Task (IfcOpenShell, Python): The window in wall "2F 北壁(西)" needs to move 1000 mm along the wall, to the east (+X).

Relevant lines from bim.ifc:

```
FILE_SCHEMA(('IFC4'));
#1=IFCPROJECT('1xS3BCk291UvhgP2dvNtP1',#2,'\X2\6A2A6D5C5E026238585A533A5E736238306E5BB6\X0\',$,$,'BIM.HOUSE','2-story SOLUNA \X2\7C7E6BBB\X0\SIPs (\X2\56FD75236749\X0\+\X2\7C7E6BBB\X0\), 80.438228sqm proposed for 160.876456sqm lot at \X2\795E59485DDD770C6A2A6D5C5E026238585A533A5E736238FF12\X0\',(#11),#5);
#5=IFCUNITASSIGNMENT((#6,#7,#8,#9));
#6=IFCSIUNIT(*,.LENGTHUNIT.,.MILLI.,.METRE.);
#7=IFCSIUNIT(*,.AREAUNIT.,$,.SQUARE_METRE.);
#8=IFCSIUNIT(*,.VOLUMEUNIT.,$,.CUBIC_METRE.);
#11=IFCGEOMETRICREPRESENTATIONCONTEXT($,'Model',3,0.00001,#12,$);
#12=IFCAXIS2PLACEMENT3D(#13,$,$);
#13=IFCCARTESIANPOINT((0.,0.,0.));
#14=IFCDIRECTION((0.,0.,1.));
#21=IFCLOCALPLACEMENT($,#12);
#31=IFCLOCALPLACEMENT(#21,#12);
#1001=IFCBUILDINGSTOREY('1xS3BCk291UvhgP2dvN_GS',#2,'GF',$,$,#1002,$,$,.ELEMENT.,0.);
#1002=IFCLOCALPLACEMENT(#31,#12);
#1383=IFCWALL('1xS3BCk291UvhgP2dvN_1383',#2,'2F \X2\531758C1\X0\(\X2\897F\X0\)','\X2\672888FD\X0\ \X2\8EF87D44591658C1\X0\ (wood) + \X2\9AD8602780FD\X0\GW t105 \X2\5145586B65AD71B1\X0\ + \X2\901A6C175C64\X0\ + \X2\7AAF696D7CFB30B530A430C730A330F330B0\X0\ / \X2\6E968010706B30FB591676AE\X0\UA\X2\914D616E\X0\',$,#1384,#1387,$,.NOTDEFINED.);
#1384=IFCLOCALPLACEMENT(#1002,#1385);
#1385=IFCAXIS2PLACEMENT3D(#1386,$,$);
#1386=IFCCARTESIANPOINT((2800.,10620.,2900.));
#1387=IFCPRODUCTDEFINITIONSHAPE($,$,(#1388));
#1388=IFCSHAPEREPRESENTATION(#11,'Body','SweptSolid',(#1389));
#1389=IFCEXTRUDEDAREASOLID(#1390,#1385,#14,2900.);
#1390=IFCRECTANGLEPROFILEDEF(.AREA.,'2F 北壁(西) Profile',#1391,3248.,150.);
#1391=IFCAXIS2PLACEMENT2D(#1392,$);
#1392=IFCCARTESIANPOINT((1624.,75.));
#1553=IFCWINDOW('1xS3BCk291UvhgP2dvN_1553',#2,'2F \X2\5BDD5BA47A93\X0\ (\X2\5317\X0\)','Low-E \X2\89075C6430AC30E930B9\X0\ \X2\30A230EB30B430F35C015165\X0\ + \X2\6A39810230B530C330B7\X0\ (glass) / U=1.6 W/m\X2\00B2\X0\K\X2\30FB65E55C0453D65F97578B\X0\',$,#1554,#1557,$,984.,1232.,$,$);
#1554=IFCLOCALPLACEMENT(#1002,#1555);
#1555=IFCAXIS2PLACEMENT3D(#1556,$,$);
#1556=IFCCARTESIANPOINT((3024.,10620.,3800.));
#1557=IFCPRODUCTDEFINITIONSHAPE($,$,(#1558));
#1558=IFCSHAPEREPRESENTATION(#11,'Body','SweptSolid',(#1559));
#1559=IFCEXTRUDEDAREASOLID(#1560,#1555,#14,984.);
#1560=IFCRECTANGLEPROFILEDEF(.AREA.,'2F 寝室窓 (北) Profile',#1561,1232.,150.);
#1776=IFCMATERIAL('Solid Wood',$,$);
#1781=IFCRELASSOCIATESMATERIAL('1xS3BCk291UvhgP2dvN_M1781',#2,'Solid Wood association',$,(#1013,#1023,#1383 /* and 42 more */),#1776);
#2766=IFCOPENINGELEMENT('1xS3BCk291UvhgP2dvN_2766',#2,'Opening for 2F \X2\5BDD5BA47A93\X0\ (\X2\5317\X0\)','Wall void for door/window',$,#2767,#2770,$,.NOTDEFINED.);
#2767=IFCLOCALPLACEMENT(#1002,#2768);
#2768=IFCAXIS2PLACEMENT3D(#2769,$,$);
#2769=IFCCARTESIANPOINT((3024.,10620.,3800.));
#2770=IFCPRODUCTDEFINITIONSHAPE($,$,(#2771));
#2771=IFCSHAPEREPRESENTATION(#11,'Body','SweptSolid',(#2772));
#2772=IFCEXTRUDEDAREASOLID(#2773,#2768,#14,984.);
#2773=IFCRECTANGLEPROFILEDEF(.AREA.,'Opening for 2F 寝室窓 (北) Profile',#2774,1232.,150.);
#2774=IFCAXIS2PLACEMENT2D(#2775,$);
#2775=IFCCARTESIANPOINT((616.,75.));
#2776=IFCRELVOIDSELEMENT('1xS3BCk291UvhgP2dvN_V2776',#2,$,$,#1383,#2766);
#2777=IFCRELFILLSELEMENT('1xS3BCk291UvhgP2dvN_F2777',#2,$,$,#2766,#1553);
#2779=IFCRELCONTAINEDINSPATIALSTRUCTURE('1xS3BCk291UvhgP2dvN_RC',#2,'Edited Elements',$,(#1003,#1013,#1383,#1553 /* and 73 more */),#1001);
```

```python
import ifcopenshell
import ifcopenshell.api.geometry
import ifcopenshell.util.placement

model = ifcopenshell.open("bim.ifc")

window = model.by_guid("1xS3BCk291UvhgP2dvN_1553")
opening = window.FillsVoids[0].RelatingOpeningElement
wall = opening.VoidsElements[0].RelatingBuildingElement

wall_matrix = ifcopenshell.util.placement.get_local_placement(wall.ObjectPlacement)
shift = wall_matrix[:3, 0] * 1000.0
before = ifcopenshell.util.placement.get_local_placement(window.ObjectPlacement)[:3, 3].copy()

# The window is not placed relative to its opening, so move both.
for product in (opening, window):
    matrix = ifcopenshell.util.placement.get_local_placement(product.ObjectPlacement)
    matrix[:3, 3] += shift
    ifcopenshell.api.geometry.edit_object_placement(model, product=product, matrix=matrix, is_si=False)

after = ifcopenshell.util.placement.get_local_placement(window.ObjectPlacement)[:3, 3]
print("window moved by", (after - before).round(3) + 0.0)

model.write("bim_rev.ifc")
```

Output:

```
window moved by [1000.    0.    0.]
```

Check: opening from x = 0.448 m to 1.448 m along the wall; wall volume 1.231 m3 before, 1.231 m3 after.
